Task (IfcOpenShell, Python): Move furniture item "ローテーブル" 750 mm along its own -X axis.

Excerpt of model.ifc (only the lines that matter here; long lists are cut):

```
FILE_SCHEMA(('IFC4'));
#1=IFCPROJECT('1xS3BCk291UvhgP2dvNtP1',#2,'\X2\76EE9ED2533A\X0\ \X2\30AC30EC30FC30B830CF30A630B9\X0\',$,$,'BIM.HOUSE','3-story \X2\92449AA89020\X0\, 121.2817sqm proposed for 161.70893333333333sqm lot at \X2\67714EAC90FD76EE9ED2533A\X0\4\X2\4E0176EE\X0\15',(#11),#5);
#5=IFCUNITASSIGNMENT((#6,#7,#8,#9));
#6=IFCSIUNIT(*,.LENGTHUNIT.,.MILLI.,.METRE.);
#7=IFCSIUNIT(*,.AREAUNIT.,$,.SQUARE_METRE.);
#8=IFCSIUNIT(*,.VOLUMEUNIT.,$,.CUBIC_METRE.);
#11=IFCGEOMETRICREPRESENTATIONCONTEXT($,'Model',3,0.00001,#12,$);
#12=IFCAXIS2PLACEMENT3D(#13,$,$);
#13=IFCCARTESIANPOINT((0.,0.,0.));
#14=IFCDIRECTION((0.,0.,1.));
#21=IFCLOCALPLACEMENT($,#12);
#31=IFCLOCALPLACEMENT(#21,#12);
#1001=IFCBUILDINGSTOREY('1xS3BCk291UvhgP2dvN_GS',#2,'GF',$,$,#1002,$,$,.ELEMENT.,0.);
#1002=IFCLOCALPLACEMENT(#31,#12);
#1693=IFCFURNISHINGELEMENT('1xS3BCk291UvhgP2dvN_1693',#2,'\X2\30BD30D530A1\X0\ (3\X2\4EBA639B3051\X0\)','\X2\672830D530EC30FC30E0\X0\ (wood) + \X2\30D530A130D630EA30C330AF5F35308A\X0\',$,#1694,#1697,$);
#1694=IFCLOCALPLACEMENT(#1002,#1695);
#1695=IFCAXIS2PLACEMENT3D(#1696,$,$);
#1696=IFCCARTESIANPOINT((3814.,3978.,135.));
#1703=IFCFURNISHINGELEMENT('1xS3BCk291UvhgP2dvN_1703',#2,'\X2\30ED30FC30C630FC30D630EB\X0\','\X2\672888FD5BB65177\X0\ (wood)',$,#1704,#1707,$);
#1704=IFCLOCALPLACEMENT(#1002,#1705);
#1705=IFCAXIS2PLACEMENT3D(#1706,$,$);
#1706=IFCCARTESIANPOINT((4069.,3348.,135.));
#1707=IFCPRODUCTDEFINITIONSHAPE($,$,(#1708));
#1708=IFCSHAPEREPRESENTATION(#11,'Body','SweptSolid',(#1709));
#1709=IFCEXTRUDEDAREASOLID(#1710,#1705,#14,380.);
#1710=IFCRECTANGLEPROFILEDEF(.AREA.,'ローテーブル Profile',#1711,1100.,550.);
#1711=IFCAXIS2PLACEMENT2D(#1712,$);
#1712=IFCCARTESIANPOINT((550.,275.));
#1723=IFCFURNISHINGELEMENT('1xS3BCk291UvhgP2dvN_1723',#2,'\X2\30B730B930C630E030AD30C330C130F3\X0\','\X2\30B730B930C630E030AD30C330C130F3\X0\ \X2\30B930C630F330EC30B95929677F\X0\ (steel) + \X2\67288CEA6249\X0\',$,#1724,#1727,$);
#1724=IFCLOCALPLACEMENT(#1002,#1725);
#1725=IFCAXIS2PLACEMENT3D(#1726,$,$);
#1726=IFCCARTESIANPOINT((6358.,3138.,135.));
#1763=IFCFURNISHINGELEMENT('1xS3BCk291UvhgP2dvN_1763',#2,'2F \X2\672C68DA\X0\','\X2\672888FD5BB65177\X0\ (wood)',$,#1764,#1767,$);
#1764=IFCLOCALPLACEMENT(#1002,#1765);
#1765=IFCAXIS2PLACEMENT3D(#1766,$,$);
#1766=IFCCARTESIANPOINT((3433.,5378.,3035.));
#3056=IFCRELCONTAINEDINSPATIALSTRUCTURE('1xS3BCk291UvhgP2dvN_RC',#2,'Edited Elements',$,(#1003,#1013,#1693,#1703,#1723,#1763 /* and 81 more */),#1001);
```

```python
import ifcopenshell
import ifcopenshell.api.geometry
import ifcopenshell.util.placement
import ifcopenshell.util.unit

model = ifcopenshell.open("model.ifc")
unit_scale = ifcopenshell.util.unit.calculate_unit_scale(model)

item = model.by_id(1703)
matrix = ifcopenshell.util.placement.get_local_placement(item.ObjectPlacement)
matrix[:3, 3] -= matrix[:3, 0] * 0.75 / unit_scale
ifcopenshell.api.geometry.edit_object_placement(model, product=item, matrix=matrix, is_si=False)

print(ifcopenshell.util.placement.get_local_placement(item.ObjectPlacement).round(3) + 0.0)

model.write("model_updated.ifc")
```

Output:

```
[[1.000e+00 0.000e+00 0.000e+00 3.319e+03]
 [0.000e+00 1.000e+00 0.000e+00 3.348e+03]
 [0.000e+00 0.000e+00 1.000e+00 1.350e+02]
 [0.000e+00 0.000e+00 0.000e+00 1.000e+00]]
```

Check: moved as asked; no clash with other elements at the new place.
